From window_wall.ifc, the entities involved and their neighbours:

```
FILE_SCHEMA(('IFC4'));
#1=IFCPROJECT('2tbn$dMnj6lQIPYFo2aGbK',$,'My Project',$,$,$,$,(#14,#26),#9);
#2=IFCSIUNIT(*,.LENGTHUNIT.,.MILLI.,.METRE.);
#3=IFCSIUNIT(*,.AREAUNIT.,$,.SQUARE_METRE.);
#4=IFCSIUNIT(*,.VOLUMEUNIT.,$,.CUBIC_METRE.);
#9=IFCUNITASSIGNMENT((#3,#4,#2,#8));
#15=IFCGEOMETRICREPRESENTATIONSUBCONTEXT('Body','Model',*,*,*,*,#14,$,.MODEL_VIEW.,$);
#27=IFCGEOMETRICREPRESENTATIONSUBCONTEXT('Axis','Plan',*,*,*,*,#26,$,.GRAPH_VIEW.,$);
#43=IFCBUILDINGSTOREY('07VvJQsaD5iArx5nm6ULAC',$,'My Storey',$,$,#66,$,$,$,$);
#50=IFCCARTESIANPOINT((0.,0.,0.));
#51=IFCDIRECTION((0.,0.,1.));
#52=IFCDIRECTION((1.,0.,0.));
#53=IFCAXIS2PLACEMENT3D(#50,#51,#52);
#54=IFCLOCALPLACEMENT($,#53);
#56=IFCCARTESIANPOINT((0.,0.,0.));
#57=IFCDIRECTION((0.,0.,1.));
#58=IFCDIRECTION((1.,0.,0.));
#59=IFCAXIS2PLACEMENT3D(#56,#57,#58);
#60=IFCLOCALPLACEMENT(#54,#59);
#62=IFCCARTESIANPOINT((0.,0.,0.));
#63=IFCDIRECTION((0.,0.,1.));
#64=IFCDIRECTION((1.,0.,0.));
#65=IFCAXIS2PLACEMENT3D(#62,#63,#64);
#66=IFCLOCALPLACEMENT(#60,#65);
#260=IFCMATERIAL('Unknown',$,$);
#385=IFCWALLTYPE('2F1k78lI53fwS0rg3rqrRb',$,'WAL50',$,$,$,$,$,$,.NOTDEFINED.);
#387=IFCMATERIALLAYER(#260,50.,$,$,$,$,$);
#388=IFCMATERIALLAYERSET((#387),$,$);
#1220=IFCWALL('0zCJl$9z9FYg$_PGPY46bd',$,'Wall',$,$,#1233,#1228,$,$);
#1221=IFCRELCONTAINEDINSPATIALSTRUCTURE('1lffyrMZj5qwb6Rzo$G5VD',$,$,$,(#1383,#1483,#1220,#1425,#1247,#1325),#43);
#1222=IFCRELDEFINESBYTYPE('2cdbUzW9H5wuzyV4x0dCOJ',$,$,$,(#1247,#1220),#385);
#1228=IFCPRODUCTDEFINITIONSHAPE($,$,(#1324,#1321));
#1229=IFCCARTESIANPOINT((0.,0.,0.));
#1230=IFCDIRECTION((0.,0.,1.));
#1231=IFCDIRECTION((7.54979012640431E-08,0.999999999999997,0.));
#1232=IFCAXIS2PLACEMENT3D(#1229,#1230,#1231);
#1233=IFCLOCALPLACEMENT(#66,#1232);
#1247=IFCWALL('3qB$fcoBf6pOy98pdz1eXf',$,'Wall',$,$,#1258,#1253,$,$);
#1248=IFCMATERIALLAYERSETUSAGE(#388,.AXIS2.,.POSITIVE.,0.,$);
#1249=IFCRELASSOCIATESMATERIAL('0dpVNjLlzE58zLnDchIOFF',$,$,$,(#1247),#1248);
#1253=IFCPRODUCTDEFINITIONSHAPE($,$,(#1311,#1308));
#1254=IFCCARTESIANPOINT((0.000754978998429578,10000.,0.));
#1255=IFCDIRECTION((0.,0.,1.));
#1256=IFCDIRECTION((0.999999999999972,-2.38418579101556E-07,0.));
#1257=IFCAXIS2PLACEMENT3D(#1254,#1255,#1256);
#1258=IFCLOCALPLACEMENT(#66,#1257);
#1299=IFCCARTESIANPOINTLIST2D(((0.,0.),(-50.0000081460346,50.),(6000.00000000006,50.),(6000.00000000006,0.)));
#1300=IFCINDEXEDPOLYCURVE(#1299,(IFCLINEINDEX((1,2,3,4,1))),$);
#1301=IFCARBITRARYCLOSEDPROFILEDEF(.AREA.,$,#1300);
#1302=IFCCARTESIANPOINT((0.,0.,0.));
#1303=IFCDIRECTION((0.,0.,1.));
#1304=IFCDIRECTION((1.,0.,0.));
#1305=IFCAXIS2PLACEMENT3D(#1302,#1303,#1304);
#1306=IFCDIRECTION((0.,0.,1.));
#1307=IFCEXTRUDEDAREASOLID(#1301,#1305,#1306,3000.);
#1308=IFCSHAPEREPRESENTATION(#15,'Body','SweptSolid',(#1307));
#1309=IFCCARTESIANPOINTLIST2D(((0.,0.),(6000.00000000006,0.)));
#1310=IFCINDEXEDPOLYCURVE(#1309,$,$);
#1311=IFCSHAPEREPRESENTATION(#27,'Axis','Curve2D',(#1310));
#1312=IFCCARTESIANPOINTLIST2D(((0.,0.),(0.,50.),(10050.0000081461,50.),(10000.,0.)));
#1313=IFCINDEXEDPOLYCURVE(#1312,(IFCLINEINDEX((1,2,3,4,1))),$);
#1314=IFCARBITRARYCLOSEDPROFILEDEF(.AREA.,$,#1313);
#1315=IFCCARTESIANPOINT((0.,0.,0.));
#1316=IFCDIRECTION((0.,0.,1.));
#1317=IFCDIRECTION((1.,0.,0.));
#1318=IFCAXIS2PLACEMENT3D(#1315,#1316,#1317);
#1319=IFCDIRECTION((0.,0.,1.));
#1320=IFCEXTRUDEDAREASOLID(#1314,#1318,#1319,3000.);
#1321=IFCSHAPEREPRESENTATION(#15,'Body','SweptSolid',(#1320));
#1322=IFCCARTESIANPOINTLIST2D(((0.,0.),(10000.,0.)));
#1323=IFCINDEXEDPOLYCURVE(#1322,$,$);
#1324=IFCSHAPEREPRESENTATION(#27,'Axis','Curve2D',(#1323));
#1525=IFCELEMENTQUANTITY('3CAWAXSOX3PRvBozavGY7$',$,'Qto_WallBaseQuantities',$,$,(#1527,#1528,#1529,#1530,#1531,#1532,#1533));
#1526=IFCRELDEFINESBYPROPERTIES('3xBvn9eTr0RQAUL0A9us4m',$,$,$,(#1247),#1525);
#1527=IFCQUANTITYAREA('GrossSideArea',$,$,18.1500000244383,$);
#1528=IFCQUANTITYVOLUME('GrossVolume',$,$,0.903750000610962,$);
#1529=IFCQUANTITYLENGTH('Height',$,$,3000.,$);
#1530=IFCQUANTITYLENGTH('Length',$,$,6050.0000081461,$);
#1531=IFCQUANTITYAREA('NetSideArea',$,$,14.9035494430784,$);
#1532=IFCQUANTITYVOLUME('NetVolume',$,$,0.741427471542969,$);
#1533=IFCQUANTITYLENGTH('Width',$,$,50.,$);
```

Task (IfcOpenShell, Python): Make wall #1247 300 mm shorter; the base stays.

```python
import ifcopenshell
import ifcopenshell.api.pset
import ifcopenshell.geom
import ifcopenshell.util.element
import ifcopenshell.util.representation
import ifcopenshell.util.shape
import ifcopenshell.util.unit

model = ifcopenshell.open("window_wall.ifc")
unit_scale = ifcopenshell.util.unit.calculate_unit_scale(model)
area_scale = ifcopenshell.util.unit.calculate_unit_scale(model, "AREAUNIT")
volume_scale = ifcopenshell.util.unit.calculate_unit_scale(model, "VOLUMEUNIT")
settings = ifcopenshell.geom.settings()


def volume(element):
    """Net volume in cubic metres, openings subtracted."""
    shape = ifcopenshell.geom.create_shape(settings, element)
    return ifcopenshell.util.shape.get_volume(shape.geometry)


wall = model.by_guid("3qB$fcoBf6pOy98pdz1eXf")
before = volume(wall)

body = ifcopenshell.util.representation.get_representation(wall, "Model", "Body")
solid = body.Items[0]
old_height = solid.Depth
solid.Depth -= 0.3 / unit_scale
after = volume(wall)
thickness = 0.05  # wall thickness in metres

# Update the stored height, areas and volumes.
qto = model.by_id(ifcopenshell.util.element.get_pset(wall, "Qto_WallBaseQuantities", should_inherit=False)["id"])
ifcopenshell.api.pset.edit_qto(model, qto=qto, properties={
    "GrossSideArea": ifcopenshell.util.element.get_pset(wall, "Qto_WallBaseQuantities", "GrossSideArea") * solid.Depth / old_height,
    "GrossVolume": ifcopenshell.util.element.get_pset(wall, "Qto_WallBaseQuantities", "GrossVolume") * solid.Depth / old_height,
    "Height": solid.Depth,
    "NetSideArea": after / thickness / area_scale,
    "NetVolume": after / volume_scale,
})

print(f"height {old_height:g} -> {solid.Depth:g}, volume {before:.3f} -> {after:.3f} m3")

model.write("window_wall-out.ifc")
```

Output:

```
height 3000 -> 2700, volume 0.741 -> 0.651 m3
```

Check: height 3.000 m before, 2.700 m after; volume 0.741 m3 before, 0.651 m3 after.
